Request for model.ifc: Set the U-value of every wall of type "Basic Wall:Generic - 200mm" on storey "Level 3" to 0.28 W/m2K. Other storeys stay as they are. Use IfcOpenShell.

First a look at what the model holds.

```python
import ifcopenshell
import ifcopenshell.util.element

model = ifcopenshell.open("model.ifc")
print(model.schema)
storey = next(s for s in model.by_type("IfcBuildingStorey") if s.Name == "Level 3")
walls = [e for e in ifcopenshell.util.element.get_decomposition(storey) if e.is_a("IfcWall")]
seen = {}
for e in walls:
    element_type = ifcopenshell.util.element.get_type(e)
    key = (element_type.Name if element_type != e and element_type else None, ifcopenshell.util.element.get_pset(e, "Pset_WallCommon", "ThermalTransmittance"))
    seen[key] = seen.get(key, 0) + 1
for (name, value), count in sorted(seen.items(), key=str):
    print(count, "x", name, "|", value)
```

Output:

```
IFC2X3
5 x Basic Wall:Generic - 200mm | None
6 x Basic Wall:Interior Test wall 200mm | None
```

```python
import ifcopenshell
import ifcopenshell.api.pset
import ifcopenshell.util.element

model = ifcopenshell.open("model.ifc")

storey = next(s for s in model.by_type("IfcBuildingStorey") if s.Name == "Level 3")
walls = [e for e in ifcopenshell.util.element.get_decomposition(storey) if e.is_a("IfcWall")]

count = 0
for e in walls:
    element_type = ifcopenshell.util.element.get_type(e)
    if element_type in (None, e) or element_type.Name != "Basic Wall:Generic - 200mm":
        continue
    # add_pset returns the element's existing set when there is one.
    pset = ifcopenshell.api.pset.add_pset(model, product=e, name="Pset_WallCommon")
    ifcopenshell.api.pset.edit_pset(model, pset=pset, properties={"ThermalTransmittance": 0.28})
    count += 1

print(count, "walls updated")

model.write("model_rev.ifc")
```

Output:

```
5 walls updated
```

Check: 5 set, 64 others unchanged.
